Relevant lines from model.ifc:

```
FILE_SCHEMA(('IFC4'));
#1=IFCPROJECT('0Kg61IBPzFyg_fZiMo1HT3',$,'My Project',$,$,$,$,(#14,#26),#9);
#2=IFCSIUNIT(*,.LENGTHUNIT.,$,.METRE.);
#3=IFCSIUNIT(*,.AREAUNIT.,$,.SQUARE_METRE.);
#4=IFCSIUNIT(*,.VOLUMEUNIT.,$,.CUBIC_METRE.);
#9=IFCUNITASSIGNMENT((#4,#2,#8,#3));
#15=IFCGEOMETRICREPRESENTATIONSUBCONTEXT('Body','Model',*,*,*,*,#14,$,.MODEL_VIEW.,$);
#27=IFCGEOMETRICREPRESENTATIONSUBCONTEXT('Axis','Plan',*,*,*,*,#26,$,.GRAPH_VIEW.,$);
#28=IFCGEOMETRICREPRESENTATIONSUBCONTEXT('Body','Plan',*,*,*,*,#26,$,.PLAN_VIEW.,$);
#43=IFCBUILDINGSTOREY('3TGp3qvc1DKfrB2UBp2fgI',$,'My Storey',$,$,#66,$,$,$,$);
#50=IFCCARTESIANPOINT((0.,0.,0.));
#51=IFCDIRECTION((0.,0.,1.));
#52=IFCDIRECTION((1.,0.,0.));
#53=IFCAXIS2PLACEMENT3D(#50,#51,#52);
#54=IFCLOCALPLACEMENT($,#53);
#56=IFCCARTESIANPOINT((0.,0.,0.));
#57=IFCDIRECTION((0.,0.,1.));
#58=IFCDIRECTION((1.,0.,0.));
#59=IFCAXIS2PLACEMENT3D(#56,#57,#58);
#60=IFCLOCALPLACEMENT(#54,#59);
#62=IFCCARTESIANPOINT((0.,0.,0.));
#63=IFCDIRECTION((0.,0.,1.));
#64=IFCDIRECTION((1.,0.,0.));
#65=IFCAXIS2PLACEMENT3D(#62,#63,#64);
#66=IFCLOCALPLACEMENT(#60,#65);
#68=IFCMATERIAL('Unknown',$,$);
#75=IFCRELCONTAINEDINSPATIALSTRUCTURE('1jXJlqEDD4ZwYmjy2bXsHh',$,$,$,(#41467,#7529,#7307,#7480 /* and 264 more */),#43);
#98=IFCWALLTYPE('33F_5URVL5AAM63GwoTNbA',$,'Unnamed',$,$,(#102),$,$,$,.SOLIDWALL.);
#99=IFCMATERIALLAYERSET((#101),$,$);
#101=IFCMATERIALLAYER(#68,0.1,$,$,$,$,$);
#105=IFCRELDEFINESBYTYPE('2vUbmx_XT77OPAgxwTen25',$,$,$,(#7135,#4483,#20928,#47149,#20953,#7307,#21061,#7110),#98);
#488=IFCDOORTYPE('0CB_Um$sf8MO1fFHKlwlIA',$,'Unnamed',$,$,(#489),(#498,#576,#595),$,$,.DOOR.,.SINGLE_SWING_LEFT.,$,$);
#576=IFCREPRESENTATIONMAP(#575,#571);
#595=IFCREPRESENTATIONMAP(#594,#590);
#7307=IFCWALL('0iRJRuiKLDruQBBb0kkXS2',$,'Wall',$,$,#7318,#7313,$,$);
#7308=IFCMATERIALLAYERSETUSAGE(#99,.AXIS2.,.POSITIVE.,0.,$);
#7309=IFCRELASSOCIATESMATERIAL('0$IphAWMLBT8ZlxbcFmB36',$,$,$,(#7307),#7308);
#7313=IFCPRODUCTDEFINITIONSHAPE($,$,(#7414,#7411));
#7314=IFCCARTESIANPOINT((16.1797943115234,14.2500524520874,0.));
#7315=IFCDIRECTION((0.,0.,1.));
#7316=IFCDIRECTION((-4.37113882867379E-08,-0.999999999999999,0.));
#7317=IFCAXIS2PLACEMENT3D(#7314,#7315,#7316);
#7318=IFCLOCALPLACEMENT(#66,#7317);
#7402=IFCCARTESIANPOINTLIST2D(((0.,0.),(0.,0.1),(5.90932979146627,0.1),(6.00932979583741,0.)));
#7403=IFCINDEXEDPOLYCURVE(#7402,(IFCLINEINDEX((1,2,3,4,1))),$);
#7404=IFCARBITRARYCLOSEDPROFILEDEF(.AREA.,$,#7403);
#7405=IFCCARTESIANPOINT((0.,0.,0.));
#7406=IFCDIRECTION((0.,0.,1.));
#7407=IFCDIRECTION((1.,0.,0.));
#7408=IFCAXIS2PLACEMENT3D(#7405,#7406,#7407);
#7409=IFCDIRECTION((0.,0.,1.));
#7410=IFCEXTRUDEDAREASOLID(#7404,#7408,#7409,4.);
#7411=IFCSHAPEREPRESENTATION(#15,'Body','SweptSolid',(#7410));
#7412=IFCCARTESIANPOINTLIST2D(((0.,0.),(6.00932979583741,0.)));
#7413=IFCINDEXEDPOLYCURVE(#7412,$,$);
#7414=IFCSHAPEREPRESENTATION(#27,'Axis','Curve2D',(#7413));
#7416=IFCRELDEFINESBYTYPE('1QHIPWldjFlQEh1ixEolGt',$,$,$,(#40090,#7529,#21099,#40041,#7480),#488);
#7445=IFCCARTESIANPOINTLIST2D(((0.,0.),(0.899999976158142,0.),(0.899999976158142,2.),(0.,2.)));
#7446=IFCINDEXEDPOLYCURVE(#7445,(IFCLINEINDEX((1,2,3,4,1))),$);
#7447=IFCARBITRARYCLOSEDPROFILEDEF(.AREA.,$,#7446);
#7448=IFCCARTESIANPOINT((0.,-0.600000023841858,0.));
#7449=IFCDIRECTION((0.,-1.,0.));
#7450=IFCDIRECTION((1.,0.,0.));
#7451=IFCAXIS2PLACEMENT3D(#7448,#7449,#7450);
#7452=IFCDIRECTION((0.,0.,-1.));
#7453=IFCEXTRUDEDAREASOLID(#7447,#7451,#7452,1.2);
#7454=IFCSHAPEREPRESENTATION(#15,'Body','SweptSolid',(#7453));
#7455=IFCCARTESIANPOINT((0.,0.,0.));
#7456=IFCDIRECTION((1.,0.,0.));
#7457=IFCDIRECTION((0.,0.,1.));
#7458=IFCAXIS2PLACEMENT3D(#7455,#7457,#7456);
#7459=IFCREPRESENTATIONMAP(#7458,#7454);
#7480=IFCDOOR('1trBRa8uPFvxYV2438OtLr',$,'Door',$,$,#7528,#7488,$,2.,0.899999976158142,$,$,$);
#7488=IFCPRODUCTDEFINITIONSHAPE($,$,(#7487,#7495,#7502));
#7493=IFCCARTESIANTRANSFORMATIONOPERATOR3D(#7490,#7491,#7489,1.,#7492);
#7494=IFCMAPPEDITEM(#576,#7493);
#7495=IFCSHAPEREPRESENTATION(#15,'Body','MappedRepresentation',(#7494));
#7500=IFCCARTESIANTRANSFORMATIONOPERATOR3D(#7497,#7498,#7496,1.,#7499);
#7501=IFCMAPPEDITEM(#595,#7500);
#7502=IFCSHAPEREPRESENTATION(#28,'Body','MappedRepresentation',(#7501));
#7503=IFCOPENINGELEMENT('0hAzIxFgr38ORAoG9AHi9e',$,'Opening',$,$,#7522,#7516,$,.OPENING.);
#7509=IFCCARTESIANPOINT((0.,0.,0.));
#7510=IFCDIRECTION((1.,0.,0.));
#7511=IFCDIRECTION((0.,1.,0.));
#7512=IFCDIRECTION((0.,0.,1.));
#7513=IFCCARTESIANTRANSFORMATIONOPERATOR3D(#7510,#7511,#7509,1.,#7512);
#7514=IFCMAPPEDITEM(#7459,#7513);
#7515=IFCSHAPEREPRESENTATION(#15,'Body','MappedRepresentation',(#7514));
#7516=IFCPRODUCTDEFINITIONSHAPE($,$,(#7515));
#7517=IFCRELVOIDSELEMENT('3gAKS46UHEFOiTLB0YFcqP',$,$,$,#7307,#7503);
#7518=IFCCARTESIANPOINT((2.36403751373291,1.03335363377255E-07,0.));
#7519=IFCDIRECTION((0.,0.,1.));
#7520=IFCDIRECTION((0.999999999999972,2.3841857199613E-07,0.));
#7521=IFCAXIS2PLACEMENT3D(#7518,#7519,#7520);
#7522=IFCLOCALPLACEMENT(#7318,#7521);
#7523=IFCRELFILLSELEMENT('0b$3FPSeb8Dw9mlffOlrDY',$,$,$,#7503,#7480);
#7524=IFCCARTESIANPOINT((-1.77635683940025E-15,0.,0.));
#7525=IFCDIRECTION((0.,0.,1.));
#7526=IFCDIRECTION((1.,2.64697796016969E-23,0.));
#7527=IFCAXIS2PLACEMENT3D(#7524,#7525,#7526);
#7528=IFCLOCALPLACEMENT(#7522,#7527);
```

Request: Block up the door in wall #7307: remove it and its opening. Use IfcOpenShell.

```python
import ifcopenshell
import ifcopenshell.api.feature
import ifcopenshell.api.root
import ifcopenshell.geom
import ifcopenshell.util.shape

model = ifcopenshell.open("model.ifc")
settings = ifcopenshell.geom.settings()


def volume(element):
    """Net volume in cubic metres, openings subtracted."""
    shape = ifcopenshell.geom.create_shape(settings, element)
    return ifcopenshell.util.shape.get_volume(shape.geometry)


door = model.by_guid("1trBRa8uPFvxYV2438OtLr")
opening = door.FillsVoids[0].RelatingOpeningElement
wall = opening.VoidsElements[0].RelatingBuildingElement
before = volume(wall)

ifcopenshell.api.root.remove_product(model, product=door)
ifcopenshell.api.feature.remove_feature(model, feature=opening)

after = volume(wall)

print(f"wall volume {before:.3f} -> {after:.3f} m3")

model.write("model_v2.ifc")
```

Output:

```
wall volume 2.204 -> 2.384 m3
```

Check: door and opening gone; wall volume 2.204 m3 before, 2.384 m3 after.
